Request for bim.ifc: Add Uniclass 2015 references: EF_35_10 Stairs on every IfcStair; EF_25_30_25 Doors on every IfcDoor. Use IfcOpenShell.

First a look at what the model holds.

```python
import ifcopenshell

model = ifcopenshell.open("bim.ifc")
print(model.schema)
print("classifications:", [c.Name for c in model.by_type("IfcClassification")])
for ifc_class in ("IfcDoor", "IfcRoof", "IfcStair", "IfcWall", "IfcWindow"):
    print(ifc_class, len(model.by_type(ifc_class)))
```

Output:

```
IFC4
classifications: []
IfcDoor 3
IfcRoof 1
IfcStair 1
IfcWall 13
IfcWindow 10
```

```python
import ifcopenshell
import ifcopenshell.api.classification

model = ifcopenshell.open("bim.ifc")

system = ifcopenshell.api.classification.add_classification(model, classification="Uniclass 2015")

codes = {
    "IfcStair": ("EF_35_10", "Stairs"),
    "IfcDoor": ("EF_25_30_25", "Doors"),
}
for ifc_class, (code, name) in codes.items():
    products = model.by_type(ifc_class)
    ifcopenshell.api.classification.add_reference(
        model, products=products, classification=system, identification=code, name=name
    )
    print(code, len(products))

model.write("bim_rev.ifc")
```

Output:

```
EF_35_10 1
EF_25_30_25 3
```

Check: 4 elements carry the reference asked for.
